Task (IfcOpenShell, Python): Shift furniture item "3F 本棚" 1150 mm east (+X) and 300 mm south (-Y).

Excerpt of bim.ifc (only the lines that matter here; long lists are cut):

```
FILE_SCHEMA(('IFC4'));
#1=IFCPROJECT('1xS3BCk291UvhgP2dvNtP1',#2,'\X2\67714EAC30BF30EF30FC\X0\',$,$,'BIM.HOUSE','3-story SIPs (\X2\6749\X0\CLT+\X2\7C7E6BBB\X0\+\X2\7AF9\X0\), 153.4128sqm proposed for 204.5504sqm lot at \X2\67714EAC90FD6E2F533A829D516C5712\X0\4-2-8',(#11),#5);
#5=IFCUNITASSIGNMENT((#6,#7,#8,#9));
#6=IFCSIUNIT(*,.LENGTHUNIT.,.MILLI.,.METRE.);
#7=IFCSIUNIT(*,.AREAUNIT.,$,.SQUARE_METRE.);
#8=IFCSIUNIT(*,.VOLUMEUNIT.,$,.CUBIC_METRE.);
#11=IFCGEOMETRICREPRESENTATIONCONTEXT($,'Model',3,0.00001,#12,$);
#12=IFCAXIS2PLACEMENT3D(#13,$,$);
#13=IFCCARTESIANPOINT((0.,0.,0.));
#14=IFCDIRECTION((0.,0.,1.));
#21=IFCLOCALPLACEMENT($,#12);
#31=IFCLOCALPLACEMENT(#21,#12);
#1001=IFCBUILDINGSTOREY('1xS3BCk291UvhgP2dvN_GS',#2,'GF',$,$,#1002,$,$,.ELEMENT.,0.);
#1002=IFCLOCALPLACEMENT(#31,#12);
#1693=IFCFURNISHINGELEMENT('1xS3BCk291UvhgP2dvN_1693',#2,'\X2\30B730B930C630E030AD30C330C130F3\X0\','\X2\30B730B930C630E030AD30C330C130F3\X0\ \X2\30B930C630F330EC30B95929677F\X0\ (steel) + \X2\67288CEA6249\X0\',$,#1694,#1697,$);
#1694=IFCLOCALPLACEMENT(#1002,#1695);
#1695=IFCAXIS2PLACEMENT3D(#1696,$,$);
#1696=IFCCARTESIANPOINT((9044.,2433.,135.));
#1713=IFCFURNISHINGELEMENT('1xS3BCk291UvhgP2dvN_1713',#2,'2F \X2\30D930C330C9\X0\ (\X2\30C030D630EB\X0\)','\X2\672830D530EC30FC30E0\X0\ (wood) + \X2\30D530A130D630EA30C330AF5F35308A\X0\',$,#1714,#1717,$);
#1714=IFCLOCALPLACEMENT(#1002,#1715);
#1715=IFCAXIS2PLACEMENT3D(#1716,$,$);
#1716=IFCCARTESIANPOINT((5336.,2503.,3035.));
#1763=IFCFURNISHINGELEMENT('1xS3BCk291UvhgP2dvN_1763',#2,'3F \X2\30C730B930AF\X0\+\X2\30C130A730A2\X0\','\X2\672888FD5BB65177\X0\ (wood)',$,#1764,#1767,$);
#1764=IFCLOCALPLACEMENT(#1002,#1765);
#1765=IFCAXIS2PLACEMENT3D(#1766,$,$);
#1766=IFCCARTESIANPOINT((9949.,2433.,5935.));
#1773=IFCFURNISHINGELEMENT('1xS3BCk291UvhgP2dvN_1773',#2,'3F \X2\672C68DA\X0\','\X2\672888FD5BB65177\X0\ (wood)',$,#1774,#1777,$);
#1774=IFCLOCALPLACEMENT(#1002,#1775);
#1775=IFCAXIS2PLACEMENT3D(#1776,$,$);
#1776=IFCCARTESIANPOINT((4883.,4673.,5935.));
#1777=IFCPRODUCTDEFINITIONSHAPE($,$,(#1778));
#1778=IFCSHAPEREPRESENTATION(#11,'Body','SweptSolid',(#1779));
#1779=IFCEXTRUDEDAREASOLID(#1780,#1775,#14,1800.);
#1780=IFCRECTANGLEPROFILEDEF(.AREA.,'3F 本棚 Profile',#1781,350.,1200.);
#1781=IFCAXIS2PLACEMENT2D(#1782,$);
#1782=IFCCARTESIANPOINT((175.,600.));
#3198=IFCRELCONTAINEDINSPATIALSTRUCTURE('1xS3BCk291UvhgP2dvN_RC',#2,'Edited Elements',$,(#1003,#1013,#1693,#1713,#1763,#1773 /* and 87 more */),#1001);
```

```python
import ifcopenshell
import ifcopenshell.api.geometry
import ifcopenshell.util.placement
import ifcopenshell.util.unit

model = ifcopenshell.open("bim.ifc")
unit_scale = ifcopenshell.util.unit.calculate_unit_scale(model)

item = model.by_guid("1xS3BCk291UvhgP2dvN_1773")
matrix = ifcopenshell.util.placement.get_local_placement(item.ObjectPlacement)
matrix[0, 3] += 1.15 / unit_scale
matrix[1, 3] -= 0.3 / unit_scale
ifcopenshell.api.geometry.edit_object_placement(model, product=item, matrix=matrix, is_si=False)

print(ifcopenshell.util.placement.get_local_placement(item.ObjectPlacement).round(3) + 0.0)

model.write("bim_rev.ifc")
```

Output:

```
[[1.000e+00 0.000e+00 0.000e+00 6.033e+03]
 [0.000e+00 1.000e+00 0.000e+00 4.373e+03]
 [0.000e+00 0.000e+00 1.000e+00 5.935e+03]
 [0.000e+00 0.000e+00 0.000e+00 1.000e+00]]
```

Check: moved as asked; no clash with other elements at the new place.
